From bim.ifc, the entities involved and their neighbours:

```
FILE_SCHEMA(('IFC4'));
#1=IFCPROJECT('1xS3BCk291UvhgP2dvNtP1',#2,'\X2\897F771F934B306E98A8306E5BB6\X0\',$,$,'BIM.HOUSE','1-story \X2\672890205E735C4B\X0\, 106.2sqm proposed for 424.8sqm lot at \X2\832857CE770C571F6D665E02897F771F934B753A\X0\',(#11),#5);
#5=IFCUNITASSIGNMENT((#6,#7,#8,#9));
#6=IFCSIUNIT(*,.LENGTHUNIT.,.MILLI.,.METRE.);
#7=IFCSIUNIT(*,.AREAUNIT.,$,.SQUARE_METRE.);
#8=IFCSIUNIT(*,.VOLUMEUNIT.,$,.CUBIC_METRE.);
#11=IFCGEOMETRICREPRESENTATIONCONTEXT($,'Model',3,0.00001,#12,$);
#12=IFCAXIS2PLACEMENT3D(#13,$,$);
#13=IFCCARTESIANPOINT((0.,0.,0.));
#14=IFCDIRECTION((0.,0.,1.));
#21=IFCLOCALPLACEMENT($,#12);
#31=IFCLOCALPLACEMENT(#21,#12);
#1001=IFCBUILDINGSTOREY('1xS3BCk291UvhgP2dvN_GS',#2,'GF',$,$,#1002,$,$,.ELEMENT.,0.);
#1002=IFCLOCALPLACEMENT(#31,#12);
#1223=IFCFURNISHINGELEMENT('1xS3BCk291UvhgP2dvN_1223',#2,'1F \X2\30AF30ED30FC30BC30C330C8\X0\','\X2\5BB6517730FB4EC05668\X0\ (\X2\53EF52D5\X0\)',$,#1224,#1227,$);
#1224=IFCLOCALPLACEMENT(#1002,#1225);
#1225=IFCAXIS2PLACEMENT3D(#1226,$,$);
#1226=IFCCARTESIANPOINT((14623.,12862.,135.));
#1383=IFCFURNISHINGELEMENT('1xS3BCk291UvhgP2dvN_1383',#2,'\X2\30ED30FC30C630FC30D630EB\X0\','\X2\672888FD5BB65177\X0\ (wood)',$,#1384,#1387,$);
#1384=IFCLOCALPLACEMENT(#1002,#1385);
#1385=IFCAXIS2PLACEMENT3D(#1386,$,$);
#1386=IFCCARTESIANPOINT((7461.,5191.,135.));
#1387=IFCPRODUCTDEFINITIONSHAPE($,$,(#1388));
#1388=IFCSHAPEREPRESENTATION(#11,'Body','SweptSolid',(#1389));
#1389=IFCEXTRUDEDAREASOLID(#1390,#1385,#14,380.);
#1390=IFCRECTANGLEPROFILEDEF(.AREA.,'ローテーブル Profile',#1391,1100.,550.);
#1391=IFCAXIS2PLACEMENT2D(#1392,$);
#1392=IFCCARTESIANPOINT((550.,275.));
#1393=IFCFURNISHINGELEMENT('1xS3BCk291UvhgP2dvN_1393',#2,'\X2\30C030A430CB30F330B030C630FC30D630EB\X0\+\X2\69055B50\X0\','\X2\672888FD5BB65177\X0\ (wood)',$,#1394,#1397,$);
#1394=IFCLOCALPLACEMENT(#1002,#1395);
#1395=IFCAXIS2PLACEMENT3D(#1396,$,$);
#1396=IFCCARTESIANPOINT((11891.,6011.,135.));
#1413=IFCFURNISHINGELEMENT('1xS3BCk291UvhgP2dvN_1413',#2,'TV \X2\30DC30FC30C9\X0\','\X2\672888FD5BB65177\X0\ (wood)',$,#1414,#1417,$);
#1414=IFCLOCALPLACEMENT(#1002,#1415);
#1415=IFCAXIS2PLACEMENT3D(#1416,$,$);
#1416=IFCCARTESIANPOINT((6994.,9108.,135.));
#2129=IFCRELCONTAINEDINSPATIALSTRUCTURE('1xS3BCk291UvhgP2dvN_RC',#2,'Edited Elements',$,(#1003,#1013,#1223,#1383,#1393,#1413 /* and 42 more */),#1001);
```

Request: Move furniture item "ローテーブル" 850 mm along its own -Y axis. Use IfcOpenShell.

```python
import ifcopenshell
import ifcopenshell.api.geometry
import ifcopenshell.util.placement
import ifcopenshell.util.unit

model = ifcopenshell.open("bim.ifc")
unit_scale = ifcopenshell.util.unit.calculate_unit_scale(model)

item = model.by_guid("1xS3BCk291UvhgP2dvN_1383")
matrix = ifcopenshell.util.placement.get_local_placement(item.ObjectPlacement)
matrix[:3, 3] -= matrix[:3, 1] * 0.85 / unit_scale
ifcopenshell.api.geometry.edit_object_placement(model, product=item, matrix=matrix, is_si=False)

print(ifcopenshell.util.placement.get_local_placement(item.ObjectPlacement).round(3) + 0.0)

model.write("bim-out.ifc")
```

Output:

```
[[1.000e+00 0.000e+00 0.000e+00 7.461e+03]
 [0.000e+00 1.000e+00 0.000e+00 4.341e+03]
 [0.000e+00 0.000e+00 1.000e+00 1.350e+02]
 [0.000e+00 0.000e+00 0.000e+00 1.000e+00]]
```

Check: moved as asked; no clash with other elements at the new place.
